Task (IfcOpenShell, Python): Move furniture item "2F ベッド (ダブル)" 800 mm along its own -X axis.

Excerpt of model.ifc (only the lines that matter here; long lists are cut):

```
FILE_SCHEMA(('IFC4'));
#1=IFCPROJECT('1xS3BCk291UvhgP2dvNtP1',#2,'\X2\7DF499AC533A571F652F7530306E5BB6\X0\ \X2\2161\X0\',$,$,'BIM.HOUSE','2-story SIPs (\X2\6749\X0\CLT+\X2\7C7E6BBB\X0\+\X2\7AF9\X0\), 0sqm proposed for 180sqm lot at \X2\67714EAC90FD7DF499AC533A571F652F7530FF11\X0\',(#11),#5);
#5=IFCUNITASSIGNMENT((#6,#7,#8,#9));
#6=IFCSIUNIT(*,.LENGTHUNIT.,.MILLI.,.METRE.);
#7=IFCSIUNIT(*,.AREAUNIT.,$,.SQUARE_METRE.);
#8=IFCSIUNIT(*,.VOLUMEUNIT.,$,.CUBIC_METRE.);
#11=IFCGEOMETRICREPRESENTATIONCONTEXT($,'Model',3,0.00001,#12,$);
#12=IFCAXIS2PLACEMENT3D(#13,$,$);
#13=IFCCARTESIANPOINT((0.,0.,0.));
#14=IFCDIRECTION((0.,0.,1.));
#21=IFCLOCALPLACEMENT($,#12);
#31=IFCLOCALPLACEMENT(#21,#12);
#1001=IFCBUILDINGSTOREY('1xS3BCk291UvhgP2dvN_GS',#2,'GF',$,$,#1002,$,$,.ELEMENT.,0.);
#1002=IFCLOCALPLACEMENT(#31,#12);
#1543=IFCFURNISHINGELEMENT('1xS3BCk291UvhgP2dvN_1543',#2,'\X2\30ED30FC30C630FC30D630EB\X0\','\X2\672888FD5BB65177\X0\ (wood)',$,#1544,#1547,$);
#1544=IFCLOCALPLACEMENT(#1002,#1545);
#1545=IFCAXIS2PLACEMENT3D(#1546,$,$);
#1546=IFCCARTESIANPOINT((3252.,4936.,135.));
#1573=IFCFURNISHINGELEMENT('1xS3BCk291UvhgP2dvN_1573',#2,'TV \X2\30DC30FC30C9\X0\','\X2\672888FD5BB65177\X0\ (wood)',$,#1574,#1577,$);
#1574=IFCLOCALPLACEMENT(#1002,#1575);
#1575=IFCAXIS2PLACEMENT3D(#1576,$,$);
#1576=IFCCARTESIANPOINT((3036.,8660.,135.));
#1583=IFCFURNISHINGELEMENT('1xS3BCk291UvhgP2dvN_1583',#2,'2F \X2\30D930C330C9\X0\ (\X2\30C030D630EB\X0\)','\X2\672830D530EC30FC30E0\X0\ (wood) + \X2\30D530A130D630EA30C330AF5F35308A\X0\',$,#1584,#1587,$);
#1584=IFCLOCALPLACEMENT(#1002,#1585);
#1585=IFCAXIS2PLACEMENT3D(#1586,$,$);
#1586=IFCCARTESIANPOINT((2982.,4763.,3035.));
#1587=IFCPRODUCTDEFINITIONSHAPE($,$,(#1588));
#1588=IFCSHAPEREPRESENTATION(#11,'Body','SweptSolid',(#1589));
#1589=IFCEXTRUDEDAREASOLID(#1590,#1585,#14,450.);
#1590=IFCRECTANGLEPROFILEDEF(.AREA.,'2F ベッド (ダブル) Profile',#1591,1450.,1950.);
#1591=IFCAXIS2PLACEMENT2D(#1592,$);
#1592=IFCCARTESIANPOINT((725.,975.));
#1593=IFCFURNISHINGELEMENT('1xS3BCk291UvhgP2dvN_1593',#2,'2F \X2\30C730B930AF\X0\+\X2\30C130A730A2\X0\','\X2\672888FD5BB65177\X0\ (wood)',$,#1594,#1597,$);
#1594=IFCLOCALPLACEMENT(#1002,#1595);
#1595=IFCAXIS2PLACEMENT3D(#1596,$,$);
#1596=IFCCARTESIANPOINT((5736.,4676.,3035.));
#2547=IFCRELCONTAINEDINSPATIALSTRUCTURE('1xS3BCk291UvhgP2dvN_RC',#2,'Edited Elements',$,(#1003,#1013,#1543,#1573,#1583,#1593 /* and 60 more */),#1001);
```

```python
import ifcopenshell
import ifcopenshell.api.geometry
import ifcopenshell.util.placement

model = ifcopenshell.open("model.ifc")

item = model.by_guid("1xS3BCk291UvhgP2dvN_1583")
matrix = ifcopenshell.util.placement.get_local_placement(item.ObjectPlacement)
matrix[:3, 3] -= matrix[:3, 0] * 800.0
ifcopenshell.api.geometry.edit_object_placement(model, product=item, matrix=matrix, is_si=False)

print(ifcopenshell.util.placement.get_local_placement(item.ObjectPlacement).round(3) + 0.0)

model.write("model_edited.ifc")
```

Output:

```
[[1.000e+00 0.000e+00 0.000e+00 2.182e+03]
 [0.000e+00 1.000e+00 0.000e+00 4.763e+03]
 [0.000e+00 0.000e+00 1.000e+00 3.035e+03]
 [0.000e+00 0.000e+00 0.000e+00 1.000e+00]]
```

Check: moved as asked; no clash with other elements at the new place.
